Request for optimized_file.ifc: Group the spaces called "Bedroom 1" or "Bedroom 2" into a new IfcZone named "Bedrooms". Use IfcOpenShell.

First a look at what the model holds.

```python
import ifcopenshell

model = ifcopenshell.open("optimized_file.ifc")
print(model.schema)
seen = {}
for space in model.by_type("IfcSpace"):
    seen[space.LongName] = seen.get(space.LongName, 0) + 1
for name, count in sorted(seen.items(), key=str):
    print(count, "x", name)
print("zones:", [z.Name for z in model.by_type("IfcZone")][:20])
```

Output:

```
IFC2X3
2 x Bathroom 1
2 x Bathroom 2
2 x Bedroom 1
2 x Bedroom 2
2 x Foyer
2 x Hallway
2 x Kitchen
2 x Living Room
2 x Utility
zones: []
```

```python
import ifcopenshell
import ifcopenshell.api.group
import ifcopenshell.api.root

model = ifcopenshell.open("optimized_file.ifc")

names = {"Bedroom 1", "Bedroom 2"}
spaces = [s for s in model.by_type("IfcSpace") if s.LongName in names]

zone = ifcopenshell.api.root.create_entity(model, ifc_class="IfcZone", name="Bedrooms")
ifcopenshell.api.group.assign_group(model, products=spaces, group=zone)
print(len(spaces), "spaces in", zone.Name)

model.write("optimized_file_v2.ifc")
```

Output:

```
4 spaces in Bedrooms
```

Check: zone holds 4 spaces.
